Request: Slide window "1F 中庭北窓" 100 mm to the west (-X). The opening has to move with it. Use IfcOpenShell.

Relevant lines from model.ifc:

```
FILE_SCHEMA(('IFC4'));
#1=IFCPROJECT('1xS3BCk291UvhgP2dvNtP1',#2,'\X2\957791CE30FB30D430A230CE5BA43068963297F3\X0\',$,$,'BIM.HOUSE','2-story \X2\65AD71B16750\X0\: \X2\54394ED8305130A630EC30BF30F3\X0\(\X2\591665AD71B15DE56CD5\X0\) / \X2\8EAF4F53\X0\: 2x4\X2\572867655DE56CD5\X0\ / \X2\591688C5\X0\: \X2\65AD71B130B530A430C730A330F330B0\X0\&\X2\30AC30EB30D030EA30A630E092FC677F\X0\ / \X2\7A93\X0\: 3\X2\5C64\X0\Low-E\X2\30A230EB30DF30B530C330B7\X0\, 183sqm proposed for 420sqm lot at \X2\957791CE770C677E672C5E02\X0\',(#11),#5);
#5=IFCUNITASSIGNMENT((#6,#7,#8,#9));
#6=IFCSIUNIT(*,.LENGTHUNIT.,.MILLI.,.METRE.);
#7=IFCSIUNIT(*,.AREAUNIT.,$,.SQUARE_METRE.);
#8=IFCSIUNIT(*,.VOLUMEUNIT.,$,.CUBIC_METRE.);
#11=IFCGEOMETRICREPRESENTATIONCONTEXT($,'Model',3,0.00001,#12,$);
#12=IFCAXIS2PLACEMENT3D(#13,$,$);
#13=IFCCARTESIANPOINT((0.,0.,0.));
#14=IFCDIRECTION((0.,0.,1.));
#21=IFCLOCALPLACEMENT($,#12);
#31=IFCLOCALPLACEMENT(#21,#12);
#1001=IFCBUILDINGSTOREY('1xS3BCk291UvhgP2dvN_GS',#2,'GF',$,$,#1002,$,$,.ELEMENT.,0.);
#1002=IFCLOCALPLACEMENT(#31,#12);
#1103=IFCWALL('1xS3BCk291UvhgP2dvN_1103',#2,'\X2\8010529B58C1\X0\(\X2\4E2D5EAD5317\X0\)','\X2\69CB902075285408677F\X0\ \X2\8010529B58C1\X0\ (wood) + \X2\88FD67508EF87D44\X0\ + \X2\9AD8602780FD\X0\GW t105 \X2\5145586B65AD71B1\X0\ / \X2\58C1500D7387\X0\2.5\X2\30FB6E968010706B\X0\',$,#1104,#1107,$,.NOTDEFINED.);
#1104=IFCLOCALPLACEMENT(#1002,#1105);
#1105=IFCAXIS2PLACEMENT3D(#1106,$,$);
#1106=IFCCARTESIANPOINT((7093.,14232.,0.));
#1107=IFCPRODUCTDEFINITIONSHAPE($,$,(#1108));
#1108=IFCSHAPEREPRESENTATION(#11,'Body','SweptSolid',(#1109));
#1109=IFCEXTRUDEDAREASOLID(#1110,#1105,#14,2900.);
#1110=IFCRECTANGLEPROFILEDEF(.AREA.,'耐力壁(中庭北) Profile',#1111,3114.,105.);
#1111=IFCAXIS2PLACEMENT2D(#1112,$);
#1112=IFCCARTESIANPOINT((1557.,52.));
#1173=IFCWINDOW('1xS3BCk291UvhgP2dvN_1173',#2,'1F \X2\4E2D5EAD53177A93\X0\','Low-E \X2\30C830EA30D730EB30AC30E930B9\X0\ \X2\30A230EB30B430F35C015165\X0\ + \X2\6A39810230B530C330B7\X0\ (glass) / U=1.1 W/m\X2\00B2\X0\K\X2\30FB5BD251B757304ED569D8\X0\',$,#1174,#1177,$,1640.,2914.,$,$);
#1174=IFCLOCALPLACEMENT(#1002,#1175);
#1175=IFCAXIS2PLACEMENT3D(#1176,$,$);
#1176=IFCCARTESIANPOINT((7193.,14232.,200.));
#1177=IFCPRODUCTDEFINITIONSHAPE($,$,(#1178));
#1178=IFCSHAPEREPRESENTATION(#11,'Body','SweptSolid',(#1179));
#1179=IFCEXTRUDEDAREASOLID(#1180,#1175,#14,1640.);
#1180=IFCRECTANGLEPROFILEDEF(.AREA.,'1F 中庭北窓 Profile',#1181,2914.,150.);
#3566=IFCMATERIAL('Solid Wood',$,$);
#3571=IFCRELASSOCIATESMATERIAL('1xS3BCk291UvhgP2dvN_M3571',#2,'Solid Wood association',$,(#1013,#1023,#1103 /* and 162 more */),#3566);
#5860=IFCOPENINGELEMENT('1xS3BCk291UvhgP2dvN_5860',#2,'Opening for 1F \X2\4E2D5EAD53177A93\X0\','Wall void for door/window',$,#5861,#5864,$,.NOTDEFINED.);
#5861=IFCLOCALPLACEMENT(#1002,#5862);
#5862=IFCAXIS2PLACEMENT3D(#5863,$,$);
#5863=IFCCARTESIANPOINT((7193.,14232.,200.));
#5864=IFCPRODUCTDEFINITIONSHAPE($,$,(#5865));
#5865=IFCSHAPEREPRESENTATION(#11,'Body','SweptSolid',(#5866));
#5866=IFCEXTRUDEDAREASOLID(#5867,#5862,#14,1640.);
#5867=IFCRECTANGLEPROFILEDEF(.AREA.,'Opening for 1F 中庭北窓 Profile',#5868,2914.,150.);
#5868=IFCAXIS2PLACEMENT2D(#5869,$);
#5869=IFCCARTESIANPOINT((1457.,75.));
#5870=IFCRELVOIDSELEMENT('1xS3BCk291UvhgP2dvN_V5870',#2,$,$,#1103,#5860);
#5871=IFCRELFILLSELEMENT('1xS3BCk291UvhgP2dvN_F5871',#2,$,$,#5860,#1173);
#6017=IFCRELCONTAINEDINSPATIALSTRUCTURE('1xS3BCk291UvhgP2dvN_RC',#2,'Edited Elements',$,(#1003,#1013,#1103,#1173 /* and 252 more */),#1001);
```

```python
import ifcopenshell
import ifcopenshell.api.geometry
import ifcopenshell.util.placement
import ifcopenshell.util.unit

model = ifcopenshell.open("model.ifc")
unit_scale = ifcopenshell.util.unit.calculate_unit_scale(model)

window = model.by_guid("1xS3BCk291UvhgP2dvN_1173")
opening = window.FillsVoids[0].RelatingOpeningElement
wall = opening.VoidsElements[0].RelatingBuildingElement

wall_matrix = ifcopenshell.util.placement.get_local_placement(wall.ObjectPlacement)
shift = wall_matrix[:3, 0] * -0.1 / unit_scale
before = ifcopenshell.util.placement.get_local_placement(window.ObjectPlacement)[:3, 3].copy()

# The window is not placed relative to its opening, so move both.
for product in (opening, window):
    matrix = ifcopenshell.util.placement.get_local_placement(product.ObjectPlacement)
    matrix[:3, 3] += shift
    ifcopenshell.api.geometry.edit_object_placement(model, product=product, matrix=matrix, is_si=False)

after = ifcopenshell.util.placement.get_local_placement(window.ObjectPlacement)[:3, 3]
print("window moved by", (after - before).round(3) + 0.0)

model.write("model_rev.ifc")
```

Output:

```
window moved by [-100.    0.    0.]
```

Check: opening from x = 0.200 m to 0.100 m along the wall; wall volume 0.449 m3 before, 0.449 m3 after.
